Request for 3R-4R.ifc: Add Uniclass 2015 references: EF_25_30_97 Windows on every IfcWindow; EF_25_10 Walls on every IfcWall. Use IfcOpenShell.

First a look at what the model holds.

```python
import ifcopenshell

model = ifcopenshell.open("3R-4R.ifc")
print(model.schema)
print("classifications:", [c.Name for c in model.by_type("IfcClassification")])
for ifc_class in ("IfcDoor", "IfcRoof", "IfcStair", "IfcWall", "IfcWindow"):
    print(ifc_class, len(model.by_type(ifc_class)))
```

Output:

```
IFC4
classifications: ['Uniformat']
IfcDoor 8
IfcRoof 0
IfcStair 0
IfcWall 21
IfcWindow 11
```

```python
import ifcopenshell
import ifcopenshell.api.classification

model = ifcopenshell.open("3R-4R.ifc")

system = ifcopenshell.api.classification.add_classification(model, classification="Uniclass 2015")

codes = {
    "IfcWindow": ("EF_25_30_97", "Windows"),
    "IfcWall": ("EF_25_10", "Walls"),
}
for ifc_class, (code, name) in codes.items():
    products = model.by_type(ifc_class)
    ifcopenshell.api.classification.add_reference(
        model, products=products, classification=system, identification=code, name=name
    )
    print(code, len(products))

model.write("3R-4R_rev.ifc")
```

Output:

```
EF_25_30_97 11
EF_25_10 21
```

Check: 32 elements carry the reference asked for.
